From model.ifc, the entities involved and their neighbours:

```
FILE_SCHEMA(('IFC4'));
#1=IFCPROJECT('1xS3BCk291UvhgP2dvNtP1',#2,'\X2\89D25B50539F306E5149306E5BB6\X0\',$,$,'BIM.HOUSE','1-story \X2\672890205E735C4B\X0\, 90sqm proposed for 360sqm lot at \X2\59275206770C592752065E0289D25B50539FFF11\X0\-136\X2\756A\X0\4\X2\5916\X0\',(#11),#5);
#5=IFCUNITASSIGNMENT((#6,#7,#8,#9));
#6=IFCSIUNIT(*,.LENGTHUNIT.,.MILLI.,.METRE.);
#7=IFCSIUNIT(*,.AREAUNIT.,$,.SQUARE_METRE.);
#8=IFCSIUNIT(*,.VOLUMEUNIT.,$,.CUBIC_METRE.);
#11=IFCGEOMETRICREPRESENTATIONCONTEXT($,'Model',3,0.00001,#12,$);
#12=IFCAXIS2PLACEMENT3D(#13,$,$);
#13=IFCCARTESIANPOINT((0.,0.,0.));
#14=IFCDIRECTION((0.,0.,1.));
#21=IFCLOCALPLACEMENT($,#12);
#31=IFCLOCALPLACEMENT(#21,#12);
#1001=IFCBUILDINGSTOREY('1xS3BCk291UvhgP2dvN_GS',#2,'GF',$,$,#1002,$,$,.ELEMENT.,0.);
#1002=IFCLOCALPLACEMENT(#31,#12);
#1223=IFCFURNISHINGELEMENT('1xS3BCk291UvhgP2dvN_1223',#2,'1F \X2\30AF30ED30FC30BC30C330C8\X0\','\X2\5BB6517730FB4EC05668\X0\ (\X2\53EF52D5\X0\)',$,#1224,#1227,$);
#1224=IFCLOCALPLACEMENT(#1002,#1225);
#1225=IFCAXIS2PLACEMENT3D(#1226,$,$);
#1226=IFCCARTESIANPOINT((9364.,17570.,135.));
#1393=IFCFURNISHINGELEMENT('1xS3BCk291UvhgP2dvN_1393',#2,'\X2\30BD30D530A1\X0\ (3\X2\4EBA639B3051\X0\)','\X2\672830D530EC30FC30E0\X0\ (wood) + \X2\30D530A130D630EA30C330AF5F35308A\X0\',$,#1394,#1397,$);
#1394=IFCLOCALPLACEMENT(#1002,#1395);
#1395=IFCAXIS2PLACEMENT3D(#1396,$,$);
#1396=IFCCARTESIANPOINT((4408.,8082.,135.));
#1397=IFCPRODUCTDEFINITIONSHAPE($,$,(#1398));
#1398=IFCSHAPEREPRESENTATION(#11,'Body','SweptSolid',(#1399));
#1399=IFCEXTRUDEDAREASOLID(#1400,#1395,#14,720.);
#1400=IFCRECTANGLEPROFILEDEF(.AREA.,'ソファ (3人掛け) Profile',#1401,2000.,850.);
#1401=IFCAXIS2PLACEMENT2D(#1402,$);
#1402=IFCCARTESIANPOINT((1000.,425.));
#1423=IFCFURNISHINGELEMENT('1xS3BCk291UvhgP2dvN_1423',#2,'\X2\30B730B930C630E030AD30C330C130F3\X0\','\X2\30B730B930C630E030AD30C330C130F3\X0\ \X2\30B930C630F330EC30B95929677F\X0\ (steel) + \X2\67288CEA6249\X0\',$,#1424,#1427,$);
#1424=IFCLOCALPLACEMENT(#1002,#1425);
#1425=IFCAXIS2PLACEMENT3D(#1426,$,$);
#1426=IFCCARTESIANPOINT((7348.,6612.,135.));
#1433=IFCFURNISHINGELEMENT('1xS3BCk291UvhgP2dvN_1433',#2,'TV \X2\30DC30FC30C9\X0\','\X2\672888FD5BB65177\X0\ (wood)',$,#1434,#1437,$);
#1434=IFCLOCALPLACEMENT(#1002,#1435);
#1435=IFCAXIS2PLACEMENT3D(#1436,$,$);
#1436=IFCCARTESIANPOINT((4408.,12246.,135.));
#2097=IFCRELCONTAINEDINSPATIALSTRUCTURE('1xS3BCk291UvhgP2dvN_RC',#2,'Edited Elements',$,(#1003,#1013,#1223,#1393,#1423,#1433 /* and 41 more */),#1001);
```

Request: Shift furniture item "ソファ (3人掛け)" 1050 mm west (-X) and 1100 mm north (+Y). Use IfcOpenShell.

```python
import ifcopenshell
import ifcopenshell.api.geometry
import ifcopenshell.util.placement
import ifcopenshell.util.unit

model = ifcopenshell.open("model.ifc")
unit_scale = ifcopenshell.util.unit.calculate_unit_scale(model)

item = model.by_guid("1xS3BCk291UvhgP2dvN_1393")
matrix = ifcopenshell.util.placement.get_local_placement(item.ObjectPlacement)
matrix[0, 3] -= 1.05 / unit_scale
matrix[1, 3] += 1.1 / unit_scale
ifcopenshell.api.geometry.edit_object_placement(model, product=item, matrix=matrix, is_si=False)

print(ifcopenshell.util.placement.get_local_placement(item.ObjectPlacement).round(3) + 0.0)

model.write("model_rev.ifc")
```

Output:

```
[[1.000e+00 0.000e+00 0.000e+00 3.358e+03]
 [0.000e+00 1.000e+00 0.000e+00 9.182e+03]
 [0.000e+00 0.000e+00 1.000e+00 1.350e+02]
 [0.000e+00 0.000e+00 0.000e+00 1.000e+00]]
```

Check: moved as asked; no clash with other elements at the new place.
